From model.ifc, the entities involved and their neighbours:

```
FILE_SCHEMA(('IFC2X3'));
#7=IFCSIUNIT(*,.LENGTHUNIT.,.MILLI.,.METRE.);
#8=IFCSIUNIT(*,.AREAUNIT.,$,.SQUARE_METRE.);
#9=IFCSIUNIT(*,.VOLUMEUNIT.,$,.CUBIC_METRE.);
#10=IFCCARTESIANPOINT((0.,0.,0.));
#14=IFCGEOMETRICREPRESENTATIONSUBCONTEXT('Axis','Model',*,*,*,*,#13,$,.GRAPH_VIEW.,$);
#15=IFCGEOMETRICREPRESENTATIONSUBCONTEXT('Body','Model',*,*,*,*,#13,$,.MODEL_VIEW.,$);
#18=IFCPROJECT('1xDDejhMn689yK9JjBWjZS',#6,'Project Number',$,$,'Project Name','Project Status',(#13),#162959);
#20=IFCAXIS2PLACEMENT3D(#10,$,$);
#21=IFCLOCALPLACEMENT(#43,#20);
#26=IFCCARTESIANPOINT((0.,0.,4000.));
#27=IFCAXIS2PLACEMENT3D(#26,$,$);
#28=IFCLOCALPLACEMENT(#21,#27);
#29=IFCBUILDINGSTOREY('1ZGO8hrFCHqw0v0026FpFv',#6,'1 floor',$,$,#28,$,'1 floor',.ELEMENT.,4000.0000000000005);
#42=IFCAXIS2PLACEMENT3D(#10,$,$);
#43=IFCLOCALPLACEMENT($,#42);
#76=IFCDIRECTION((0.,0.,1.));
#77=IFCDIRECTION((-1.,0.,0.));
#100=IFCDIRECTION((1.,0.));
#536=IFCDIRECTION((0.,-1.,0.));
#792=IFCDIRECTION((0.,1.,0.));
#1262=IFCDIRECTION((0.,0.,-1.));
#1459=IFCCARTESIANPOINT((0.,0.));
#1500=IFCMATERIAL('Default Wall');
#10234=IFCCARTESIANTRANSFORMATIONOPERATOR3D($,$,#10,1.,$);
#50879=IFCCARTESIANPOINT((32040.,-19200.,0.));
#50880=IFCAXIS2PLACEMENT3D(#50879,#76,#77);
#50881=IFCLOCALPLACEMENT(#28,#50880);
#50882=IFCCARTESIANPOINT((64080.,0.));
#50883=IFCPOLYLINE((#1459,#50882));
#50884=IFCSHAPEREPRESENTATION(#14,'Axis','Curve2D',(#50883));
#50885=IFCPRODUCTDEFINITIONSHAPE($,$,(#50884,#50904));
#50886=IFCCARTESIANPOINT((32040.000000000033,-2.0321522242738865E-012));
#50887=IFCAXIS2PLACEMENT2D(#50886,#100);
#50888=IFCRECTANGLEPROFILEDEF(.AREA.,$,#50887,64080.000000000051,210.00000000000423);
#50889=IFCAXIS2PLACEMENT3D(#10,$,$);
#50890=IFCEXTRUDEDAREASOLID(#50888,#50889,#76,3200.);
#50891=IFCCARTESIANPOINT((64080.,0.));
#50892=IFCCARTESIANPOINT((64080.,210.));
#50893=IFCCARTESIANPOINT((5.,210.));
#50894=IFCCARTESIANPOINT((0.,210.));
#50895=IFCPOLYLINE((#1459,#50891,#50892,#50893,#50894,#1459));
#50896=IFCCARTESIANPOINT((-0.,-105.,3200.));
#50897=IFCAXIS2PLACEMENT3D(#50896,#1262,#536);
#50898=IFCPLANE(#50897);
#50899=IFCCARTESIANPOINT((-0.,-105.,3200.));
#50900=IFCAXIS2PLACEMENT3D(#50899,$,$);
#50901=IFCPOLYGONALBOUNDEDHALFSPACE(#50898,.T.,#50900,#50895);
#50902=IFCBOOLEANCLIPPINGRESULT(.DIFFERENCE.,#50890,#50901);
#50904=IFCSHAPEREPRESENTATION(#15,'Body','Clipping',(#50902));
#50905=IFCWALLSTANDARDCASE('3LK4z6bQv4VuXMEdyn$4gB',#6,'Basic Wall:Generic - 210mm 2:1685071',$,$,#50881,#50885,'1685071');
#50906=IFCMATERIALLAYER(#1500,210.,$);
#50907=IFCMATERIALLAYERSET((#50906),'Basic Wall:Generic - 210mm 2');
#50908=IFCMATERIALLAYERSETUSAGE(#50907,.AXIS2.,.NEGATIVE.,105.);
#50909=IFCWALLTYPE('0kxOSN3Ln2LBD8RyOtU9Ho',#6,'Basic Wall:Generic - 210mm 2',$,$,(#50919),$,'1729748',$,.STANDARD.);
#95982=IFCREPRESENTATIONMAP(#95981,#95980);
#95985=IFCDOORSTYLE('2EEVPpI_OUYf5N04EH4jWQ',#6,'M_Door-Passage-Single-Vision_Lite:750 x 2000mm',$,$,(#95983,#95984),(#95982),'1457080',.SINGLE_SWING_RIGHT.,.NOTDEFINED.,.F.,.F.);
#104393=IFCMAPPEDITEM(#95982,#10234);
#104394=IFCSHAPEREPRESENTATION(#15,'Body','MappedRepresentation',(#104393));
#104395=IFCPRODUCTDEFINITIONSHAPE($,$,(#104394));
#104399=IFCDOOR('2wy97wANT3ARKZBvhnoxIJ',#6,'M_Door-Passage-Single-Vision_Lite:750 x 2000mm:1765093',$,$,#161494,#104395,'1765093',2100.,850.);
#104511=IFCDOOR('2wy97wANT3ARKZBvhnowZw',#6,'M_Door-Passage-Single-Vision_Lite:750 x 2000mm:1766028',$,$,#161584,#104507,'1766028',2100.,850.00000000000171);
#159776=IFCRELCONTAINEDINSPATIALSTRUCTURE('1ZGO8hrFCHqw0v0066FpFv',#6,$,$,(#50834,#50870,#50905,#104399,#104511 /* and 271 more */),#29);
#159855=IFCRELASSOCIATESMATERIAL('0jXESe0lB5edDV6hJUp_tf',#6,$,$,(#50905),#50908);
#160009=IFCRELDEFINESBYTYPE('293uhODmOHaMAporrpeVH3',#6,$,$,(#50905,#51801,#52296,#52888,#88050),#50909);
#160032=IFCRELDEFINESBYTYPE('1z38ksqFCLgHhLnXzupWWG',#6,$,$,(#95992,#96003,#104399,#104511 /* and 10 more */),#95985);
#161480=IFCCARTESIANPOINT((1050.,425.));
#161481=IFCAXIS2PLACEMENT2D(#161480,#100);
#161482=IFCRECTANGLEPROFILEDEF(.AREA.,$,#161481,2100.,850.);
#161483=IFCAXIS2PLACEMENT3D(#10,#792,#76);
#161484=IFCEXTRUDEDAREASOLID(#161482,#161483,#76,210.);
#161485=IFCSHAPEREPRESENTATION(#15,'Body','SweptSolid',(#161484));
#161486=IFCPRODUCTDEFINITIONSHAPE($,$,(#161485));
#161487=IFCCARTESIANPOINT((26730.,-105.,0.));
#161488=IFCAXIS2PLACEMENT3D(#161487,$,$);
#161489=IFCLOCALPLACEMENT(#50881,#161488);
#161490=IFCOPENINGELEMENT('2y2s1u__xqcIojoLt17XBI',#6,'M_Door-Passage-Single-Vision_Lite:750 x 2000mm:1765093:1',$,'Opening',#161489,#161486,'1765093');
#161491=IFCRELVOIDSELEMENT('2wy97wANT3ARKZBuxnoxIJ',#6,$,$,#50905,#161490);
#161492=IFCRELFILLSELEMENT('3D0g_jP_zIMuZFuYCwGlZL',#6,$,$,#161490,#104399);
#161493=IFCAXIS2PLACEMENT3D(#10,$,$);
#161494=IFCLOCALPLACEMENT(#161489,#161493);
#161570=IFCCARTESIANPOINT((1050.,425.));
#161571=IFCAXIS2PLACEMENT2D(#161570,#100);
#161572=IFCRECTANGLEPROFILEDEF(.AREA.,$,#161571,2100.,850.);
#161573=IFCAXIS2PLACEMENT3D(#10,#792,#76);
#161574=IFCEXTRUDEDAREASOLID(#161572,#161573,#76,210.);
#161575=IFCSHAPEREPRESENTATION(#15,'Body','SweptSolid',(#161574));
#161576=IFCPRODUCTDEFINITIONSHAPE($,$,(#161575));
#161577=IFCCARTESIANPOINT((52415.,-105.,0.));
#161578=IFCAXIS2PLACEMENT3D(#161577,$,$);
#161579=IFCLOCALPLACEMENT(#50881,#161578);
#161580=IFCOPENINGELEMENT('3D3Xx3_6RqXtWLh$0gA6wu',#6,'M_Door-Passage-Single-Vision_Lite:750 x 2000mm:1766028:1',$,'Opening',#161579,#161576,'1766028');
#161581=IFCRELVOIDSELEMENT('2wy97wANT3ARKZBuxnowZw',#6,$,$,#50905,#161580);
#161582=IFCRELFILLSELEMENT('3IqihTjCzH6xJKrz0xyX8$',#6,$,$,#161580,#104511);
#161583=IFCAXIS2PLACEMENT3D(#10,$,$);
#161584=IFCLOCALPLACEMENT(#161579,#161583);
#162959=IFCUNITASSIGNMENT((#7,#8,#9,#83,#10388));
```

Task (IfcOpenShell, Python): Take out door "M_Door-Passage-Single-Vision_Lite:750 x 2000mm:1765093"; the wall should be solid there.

```python
import ifcopenshell
import ifcopenshell.api.feature
import ifcopenshell.api.root
import ifcopenshell.geom
import ifcopenshell.util.shape

model = ifcopenshell.open("model.ifc")
settings = ifcopenshell.geom.settings()


def volume(element):
    """Net volume in cubic metres, openings subtracted."""
    shape = ifcopenshell.geom.create_shape(settings, element)
    return ifcopenshell.util.shape.get_volume(shape.geometry)


door = model.by_guid("2wy97wANT3ARKZBvhnoxIJ")
opening = door.FillsVoids[0].RelatingOpeningElement
wall = opening.VoidsElements[0].RelatingBuildingElement
before = volume(wall)

ifcopenshell.api.root.remove_product(model, product=door)
ifcopenshell.api.feature.remove_feature(model, feature=opening)

after = volume(wall)

print(f"wall volume {before:.3f} -> {after:.3f} m3")

model.write("model_edited.ifc")
```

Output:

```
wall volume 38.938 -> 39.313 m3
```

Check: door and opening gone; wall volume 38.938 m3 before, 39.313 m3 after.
